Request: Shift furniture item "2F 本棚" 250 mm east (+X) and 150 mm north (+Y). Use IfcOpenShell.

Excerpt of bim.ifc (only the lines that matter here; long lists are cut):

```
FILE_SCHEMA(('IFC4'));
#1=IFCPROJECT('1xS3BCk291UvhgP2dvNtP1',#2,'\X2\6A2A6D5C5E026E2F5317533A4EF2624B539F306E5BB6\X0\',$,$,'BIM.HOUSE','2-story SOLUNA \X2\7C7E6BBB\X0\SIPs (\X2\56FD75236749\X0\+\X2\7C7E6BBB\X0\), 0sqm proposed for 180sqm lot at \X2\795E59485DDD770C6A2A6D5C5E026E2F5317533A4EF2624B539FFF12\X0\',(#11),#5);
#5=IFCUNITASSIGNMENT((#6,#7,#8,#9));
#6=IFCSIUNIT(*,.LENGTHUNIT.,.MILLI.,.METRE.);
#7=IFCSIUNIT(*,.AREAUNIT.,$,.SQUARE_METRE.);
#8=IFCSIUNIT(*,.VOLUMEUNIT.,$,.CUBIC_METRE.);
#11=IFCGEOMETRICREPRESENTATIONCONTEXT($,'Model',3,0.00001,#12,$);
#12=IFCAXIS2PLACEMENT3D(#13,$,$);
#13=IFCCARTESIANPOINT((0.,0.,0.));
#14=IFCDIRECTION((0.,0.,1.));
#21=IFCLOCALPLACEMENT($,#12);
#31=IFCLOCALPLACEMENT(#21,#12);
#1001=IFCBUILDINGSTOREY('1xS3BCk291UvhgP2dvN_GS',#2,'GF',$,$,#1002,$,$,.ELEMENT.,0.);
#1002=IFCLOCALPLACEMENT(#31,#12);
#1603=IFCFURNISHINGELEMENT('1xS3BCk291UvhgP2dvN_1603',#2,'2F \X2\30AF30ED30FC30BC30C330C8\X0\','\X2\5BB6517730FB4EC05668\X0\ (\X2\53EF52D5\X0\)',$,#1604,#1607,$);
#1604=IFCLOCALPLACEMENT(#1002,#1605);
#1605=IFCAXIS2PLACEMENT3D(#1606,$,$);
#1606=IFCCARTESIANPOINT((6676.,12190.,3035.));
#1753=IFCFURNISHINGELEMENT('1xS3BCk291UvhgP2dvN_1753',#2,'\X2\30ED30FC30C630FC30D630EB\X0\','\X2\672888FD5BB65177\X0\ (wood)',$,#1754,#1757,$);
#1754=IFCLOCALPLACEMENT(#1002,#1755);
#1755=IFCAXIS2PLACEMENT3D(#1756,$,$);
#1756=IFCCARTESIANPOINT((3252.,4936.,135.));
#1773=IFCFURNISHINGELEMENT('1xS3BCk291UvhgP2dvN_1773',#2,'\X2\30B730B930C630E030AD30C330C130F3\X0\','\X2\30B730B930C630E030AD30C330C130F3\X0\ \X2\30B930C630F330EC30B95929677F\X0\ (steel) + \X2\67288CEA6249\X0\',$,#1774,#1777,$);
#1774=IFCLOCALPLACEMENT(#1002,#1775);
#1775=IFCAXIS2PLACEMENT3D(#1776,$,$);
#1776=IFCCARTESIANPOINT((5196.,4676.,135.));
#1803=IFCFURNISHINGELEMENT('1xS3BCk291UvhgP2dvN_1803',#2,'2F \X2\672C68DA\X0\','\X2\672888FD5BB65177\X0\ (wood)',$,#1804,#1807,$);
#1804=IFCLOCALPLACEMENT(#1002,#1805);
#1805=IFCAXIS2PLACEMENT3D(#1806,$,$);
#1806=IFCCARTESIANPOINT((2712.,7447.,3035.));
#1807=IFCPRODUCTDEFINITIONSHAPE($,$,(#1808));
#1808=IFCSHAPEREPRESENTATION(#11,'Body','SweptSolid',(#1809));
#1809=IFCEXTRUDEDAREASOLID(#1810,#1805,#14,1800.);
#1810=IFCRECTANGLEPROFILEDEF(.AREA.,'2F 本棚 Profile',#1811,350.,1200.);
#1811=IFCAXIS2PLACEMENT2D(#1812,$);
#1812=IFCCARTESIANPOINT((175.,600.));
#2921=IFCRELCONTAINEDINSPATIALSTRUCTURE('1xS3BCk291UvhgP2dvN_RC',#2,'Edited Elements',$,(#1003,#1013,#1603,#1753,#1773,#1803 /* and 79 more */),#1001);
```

```python
import ifcopenshell
import ifcopenshell.api.geometry
import ifcopenshell.util.placement
import ifcopenshell.util.unit

model = ifcopenshell.open("bim.ifc")
unit_scale = ifcopenshell.util.unit.calculate_unit_scale(model)

item = model.by_id(1803)
matrix = ifcopenshell.util.placement.get_local_placement(item.ObjectPlacement)
matrix[0, 3] += 0.25 / unit_scale
matrix[1, 3] += 0.15 / unit_scale
ifcopenshell.api.geometry.edit_object_placement(model, product=item, matrix=matrix, is_si=False)

print(ifcopenshell.util.placement.get_local_placement(item.ObjectPlacement).round(3) + 0.0)

model.write("bim-out.ifc")
```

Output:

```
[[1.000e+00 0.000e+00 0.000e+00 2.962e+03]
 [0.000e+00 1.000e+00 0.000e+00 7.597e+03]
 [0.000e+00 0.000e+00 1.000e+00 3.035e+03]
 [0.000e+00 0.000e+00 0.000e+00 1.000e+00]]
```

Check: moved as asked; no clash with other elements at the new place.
